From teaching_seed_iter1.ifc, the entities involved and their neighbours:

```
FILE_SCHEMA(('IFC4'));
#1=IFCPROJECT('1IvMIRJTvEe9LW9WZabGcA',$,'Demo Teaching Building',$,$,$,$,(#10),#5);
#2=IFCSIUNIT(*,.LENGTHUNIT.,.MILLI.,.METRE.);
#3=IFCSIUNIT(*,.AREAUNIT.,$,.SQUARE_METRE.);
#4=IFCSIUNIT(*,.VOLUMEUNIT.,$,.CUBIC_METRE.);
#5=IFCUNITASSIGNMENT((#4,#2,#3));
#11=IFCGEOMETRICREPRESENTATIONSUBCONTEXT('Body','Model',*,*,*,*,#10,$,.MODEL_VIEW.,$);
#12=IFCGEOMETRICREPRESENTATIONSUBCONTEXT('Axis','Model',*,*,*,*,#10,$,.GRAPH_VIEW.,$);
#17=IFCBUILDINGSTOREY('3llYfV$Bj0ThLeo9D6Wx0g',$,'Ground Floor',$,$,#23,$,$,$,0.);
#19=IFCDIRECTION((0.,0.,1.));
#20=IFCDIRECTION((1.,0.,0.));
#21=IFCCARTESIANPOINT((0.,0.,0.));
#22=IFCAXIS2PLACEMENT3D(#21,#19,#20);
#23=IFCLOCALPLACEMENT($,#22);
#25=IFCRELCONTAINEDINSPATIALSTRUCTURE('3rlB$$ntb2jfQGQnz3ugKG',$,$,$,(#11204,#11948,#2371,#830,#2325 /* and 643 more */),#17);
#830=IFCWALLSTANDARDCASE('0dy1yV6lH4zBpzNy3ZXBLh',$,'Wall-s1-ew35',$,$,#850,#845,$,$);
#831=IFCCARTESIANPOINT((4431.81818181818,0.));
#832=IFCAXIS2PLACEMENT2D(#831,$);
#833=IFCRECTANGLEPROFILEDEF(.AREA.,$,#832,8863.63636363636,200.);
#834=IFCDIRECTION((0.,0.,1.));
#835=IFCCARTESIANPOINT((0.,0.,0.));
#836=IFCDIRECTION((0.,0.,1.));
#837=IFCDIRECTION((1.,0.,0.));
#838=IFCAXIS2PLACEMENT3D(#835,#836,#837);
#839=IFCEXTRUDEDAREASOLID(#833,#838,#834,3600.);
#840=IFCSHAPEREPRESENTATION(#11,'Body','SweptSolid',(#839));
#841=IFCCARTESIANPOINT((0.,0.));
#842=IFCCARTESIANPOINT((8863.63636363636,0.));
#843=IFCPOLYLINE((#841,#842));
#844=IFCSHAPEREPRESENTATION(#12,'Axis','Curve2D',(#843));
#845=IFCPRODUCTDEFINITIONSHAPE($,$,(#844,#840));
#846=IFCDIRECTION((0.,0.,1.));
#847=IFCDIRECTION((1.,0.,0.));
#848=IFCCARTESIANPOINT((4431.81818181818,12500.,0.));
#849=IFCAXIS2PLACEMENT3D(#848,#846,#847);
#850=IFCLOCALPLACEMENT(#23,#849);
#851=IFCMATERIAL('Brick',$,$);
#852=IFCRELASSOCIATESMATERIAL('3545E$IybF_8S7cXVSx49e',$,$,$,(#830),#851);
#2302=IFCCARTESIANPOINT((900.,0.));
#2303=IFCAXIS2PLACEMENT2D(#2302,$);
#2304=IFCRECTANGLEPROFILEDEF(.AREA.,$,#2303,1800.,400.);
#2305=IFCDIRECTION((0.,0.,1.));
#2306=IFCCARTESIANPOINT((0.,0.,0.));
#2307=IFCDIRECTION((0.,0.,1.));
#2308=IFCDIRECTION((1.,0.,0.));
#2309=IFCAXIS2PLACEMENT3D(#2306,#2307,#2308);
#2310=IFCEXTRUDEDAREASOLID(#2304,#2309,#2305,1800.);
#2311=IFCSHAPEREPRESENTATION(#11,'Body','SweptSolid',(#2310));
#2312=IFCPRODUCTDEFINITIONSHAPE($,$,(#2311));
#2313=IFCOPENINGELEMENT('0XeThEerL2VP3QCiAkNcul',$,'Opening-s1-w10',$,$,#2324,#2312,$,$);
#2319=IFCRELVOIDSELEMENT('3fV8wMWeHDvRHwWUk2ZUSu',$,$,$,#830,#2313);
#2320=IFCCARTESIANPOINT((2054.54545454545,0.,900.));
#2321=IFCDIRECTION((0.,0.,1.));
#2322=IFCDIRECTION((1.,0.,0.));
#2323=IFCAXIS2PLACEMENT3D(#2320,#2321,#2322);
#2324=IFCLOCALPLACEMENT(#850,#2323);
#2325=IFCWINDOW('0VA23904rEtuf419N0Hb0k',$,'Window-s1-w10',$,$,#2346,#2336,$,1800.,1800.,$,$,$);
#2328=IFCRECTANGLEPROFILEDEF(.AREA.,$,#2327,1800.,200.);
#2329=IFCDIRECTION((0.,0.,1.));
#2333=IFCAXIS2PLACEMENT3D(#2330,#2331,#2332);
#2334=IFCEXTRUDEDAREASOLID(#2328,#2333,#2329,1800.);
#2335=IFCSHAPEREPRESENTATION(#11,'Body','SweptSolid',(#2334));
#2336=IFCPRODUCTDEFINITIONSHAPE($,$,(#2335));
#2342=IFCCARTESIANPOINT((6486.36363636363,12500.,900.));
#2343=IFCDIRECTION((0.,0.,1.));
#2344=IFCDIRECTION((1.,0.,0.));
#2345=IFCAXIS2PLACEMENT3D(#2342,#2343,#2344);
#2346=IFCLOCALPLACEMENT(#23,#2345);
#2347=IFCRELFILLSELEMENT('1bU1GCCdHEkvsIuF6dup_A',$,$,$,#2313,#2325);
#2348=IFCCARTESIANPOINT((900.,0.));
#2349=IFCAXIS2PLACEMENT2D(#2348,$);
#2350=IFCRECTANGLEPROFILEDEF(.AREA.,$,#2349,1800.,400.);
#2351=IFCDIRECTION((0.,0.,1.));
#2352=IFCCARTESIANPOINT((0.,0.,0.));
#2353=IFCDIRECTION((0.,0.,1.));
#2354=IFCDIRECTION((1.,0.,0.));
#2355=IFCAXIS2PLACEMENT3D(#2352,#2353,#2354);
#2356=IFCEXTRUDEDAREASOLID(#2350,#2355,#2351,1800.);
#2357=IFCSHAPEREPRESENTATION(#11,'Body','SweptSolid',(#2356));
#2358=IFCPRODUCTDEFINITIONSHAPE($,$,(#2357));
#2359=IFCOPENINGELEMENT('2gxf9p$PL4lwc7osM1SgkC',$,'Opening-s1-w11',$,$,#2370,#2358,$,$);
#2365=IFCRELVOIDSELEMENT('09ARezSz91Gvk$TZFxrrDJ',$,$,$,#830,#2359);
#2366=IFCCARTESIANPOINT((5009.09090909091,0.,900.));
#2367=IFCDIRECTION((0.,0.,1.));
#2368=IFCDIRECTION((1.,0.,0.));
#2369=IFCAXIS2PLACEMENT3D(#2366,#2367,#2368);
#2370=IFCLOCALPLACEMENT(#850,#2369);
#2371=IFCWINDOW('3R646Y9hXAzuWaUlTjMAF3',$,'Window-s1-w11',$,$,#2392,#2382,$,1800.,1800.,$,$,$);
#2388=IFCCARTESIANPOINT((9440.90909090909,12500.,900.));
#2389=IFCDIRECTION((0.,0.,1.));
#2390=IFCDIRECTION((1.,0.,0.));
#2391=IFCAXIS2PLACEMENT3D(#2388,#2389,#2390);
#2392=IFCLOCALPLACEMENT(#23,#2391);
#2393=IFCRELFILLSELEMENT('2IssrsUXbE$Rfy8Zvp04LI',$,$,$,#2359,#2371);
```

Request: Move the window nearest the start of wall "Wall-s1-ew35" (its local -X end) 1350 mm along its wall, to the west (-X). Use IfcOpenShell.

```python
import ifcopenshell
import ifcopenshell.api.geometry
import ifcopenshell.util.placement
import ifcopenshell.util.unit

model = ifcopenshell.open("teaching_seed_iter1.ifc")
unit_scale = ifcopenshell.util.unit.calculate_unit_scale(model)

window = model.by_guid("0VA23904rEtuf419N0Hb0k")
opening = window.FillsVoids[0].RelatingOpeningElement
wall = opening.VoidsElements[0].RelatingBuildingElement

wall_matrix = ifcopenshell.util.placement.get_local_placement(wall.ObjectPlacement)
shift = wall_matrix[:3, 0] * -1.35 / unit_scale
before = ifcopenshell.util.placement.get_local_placement(window.ObjectPlacement)[:3, 3].copy()

# The window is not placed relative to its opening, so move both.
for product in (opening, window):
    matrix = ifcopenshell.util.placement.get_local_placement(product.ObjectPlacement)
    matrix[:3, 3] += shift
    ifcopenshell.api.geometry.edit_object_placement(model, product=product, matrix=matrix, is_si=False)

after = ifcopenshell.util.placement.get_local_placement(window.ObjectPlacement)[:3, 3]
print("window moved by", (after - before).round(3) + 0.0)

model.write("teaching_seed_iter1-out.ifc")
```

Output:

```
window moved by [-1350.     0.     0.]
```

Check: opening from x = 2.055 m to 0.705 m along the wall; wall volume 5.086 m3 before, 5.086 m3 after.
